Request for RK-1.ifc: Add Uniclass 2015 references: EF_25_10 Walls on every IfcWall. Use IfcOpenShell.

First a look at what the model holds.

```python
import ifcopenshell

model = ifcopenshell.open("RK-1.ifc")
print(model.schema)
print("classifications:", [c.Name for c in model.by_type("IfcClassification")])
for ifc_class in ("IfcDoor", "IfcRoof", "IfcStair", "IfcWall", "IfcWindow"):
    print(ifc_class, len(model.by_type(ifc_class)))
```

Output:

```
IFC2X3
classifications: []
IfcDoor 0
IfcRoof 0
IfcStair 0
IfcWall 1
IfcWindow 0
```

```python
import ifcopenshell
import ifcopenshell.api.classification

model = ifcopenshell.open("RK-1.ifc")

# IFC2X3 requires Source and Edition and has no link from the project to the system.
system = model.create_entity("IfcClassification", Source="NBS", Edition="2015", Name="Uniclass 2015")

codes = {
    "IfcWall": ("EF_25_10", "Walls"),
}
for ifc_class, (code, name) in codes.items():
    products = model.by_type(ifc_class)
    ifcopenshell.api.classification.add_reference(
        model, products=products, classification=system, identification=code, name=name
    )
    print(code, len(products))

model.write("RK-1_rev.ifc")
```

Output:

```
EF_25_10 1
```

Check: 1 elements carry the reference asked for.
